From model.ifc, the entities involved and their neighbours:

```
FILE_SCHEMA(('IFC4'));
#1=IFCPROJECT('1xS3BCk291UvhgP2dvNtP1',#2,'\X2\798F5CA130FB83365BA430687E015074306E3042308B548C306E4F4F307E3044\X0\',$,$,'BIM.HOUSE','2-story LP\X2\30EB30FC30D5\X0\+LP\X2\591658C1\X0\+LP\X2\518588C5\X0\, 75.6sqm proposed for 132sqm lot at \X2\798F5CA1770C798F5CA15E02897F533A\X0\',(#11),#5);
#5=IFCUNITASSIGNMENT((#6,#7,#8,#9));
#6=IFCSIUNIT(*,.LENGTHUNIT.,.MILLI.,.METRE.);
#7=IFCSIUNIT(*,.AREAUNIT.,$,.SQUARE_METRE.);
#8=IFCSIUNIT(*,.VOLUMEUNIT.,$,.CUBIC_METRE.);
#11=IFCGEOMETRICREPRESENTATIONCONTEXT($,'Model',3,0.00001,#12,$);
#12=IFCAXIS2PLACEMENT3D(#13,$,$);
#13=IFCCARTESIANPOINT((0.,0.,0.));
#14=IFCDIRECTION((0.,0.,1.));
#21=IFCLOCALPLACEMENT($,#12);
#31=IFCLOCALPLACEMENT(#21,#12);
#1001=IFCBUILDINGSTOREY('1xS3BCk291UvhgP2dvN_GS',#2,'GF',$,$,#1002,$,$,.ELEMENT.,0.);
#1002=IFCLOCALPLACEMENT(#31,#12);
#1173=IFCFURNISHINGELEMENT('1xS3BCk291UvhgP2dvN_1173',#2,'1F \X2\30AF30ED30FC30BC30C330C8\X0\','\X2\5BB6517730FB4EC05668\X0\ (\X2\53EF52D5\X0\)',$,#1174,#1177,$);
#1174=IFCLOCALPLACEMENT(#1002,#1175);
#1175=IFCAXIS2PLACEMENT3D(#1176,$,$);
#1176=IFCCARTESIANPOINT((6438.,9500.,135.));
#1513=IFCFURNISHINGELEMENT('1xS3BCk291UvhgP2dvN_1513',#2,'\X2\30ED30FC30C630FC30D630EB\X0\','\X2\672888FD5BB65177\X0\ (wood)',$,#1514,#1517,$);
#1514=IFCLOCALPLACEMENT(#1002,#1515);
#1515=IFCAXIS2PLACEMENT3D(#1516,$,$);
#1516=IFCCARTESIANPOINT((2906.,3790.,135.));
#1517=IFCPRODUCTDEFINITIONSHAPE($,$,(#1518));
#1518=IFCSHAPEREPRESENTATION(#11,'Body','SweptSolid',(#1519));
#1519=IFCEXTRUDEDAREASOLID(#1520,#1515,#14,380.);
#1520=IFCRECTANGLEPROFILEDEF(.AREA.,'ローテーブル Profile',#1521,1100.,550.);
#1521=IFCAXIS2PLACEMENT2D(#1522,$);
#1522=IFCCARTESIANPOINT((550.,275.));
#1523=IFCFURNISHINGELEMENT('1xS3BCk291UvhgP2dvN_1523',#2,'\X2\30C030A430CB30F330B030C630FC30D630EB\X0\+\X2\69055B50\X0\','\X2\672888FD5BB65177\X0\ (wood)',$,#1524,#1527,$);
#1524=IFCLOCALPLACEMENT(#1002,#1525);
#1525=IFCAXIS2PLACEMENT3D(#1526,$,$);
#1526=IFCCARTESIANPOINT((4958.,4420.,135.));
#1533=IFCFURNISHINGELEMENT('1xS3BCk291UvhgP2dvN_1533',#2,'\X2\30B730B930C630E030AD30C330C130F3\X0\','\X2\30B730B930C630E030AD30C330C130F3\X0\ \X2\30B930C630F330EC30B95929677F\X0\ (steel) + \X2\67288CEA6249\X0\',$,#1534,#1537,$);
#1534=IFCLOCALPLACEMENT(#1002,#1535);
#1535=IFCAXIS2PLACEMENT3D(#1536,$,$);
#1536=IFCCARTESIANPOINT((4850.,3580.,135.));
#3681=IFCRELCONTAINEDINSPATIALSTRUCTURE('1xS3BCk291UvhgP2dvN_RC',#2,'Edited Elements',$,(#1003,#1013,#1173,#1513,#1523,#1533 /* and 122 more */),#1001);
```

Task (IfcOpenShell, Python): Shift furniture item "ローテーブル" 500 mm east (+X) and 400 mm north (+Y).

```python
import ifcopenshell
import ifcopenshell.api.geometry
import ifcopenshell.util.placement
import ifcopenshell.util.unit

model = ifcopenshell.open("model.ifc")
unit_scale = ifcopenshell.util.unit.calculate_unit_scale(model)

item = model.by_guid("1xS3BCk291UvhgP2dvN_1513")
matrix = ifcopenshell.util.placement.get_local_placement(item.ObjectPlacement)
matrix[0, 3] += 0.5 / unit_scale
matrix[1, 3] += 0.4 / unit_scale
ifcopenshell.api.geometry.edit_object_placement(model, product=item, matrix=matrix, is_si=False)

print(ifcopenshell.util.placement.get_local_placement(item.ObjectPlacement).round(3) + 0.0)

model.write("model_rev.ifc")
```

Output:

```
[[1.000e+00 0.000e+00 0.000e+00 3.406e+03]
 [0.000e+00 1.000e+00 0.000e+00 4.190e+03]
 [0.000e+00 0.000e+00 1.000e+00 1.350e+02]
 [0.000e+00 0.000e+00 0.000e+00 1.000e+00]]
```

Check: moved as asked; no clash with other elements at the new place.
